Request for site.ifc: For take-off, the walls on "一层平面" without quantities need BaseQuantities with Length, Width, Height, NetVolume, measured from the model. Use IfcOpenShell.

First a look at what the model holds.

```python
import ifcopenshell
import ifcopenshell.util.element
import ifcopenshell.util.unit

model = ifcopenshell.open("site.ifc")
print(model.schema)
for unit_type in ("LENGTHUNIT", "AREAUNIT", "VOLUMEUNIT"):
    print(unit_type, ifcopenshell.util.unit.calculate_unit_scale(model, unit_type))
storey = next(s for s in model.by_type("IfcBuildingStorey") if s.Name == "一层平面")
walls = [e for e in ifcopenshell.util.element.get_decomposition(storey) if e.is_a("IfcWall")]
for e in sorted(walls, key=lambda e: e.id()):
    print(e.id(), e.is_a(), e.Name, list(ifcopenshell.util.element.get_psets(e, qtos_only=True)), sep=" | ")
```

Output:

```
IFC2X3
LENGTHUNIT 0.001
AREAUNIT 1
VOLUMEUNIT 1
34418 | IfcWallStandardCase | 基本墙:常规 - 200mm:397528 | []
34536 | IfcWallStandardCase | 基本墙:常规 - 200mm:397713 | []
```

```python
import ifcopenshell
import ifcopenshell.api.pset
import ifcopenshell.geom
import ifcopenshell.util.element
import ifcopenshell.util.shape
import ifcopenshell.util.unit

model = ifcopenshell.open("site.ifc")
unit_scale = ifcopenshell.util.unit.calculate_unit_scale(model)
volume_scale = ifcopenshell.util.unit.calculate_unit_scale(model, "VOLUMEUNIT")
settings = ifcopenshell.geom.settings()

storey = next(s for s in model.by_type("IfcBuildingStorey") if s.Name == "一层平面")
walls = [e for e in ifcopenshell.util.element.get_decomposition(storey) if e.is_a("IfcWall")]

for e in sorted(walls, key=lambda e: e.id()):
    if ifcopenshell.util.element.get_psets(e, qtos_only=True, should_inherit=False):
        continue
    # Geometry comes back in metres, in the element's own axes.
    shape = ifcopenshell.geom.create_shape(settings, e)
    values = {
        "Length": ifcopenshell.util.shape.get_x(shape.geometry) / unit_scale,
        "Width": ifcopenshell.util.shape.get_y(shape.geometry) / unit_scale,
        "Height": ifcopenshell.util.shape.get_z(shape.geometry) / unit_scale,
        "NetVolume": ifcopenshell.util.shape.get_volume(shape.geometry) / volume_scale,
    }
    qto = ifcopenshell.api.pset.add_qto(model, product=e, name="BaseQuantities")
    ifcopenshell.api.pset.edit_qto(model, qto=qto, properties=values)
    print(e.id(), {k: round(v, 3) for k, v in values.items()})

model.write("site_rev.ifc")
```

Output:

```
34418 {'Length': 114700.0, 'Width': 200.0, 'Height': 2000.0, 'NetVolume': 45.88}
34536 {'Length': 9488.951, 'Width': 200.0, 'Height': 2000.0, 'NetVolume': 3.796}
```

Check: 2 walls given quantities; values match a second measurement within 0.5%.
